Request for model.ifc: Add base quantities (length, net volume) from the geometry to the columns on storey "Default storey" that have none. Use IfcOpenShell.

First a look at what the model holds.

```python
import ifcopenshell
import ifcopenshell.util.element
import ifcopenshell.util.unit

model = ifcopenshell.open("model.ifc")
print(model.schema)
for unit_type in ("LENGTHUNIT", "AREAUNIT", "VOLUMEUNIT"):
    print(unit_type, ifcopenshell.util.unit.calculate_unit_scale(model, unit_type))
storey = next(s for s in model.by_type("IfcBuildingStorey") if s.Name == "Default storey")
columns = [e for e in ifcopenshell.util.element.get_decomposition(storey) if e.is_a("IfcColumn")]
for e in sorted(columns, key=lambda e: e.id()):
    print(e.id(), e.is_a(), e.Name, list(ifcopenshell.util.element.get_psets(e, qtos_only=True)), sep=" | ")
```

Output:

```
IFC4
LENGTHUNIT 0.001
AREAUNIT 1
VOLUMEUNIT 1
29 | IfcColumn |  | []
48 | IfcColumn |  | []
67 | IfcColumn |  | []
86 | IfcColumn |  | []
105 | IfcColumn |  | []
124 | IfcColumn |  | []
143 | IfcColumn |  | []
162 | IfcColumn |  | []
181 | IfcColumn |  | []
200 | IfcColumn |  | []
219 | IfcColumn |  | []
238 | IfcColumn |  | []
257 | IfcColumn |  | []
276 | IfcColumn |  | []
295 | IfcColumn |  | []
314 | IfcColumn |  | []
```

```python
import ifcopenshell
import ifcopenshell.api.pset
import ifcopenshell.geom
import ifcopenshell.util.element
import ifcopenshell.util.shape
import ifcopenshell.util.unit

model = ifcopenshell.open("model.ifc")
unit_scale = ifcopenshell.util.unit.calculate_unit_scale(model)
volume_scale = ifcopenshell.util.unit.calculate_unit_scale(model, "VOLUMEUNIT")
settings = ifcopenshell.geom.settings()

storey = next(s for s in model.by_type("IfcBuildingStorey") if s.Name == "Default storey")
columns = [e for e in ifcopenshell.util.element.get_decomposition(storey) if e.is_a("IfcColumn")]

for e in sorted(columns, key=lambda e: e.id()):
    if ifcopenshell.util.element.get_psets(e, qtos_only=True, should_inherit=False):
        continue
    # Geometry comes back in metres, in the element's own axes.
    shape = ifcopenshell.geom.create_shape(settings, e)
    values = {
        "Length": ifcopenshell.util.shape.get_z(shape.geometry) / unit_scale,
        "NetVolume": ifcopenshell.util.shape.get_volume(shape.geometry) / volume_scale,
    }
    qto = ifcopenshell.api.pset.add_qto(model, product=e, name="Qto_ColumnBaseQuantities")
    ifcopenshell.api.pset.edit_qto(model, qto=qto, properties=values)
    print(e.id(), {k: round(v, 3) for k, v in values.items()})

model.write("model-out.ifc")
```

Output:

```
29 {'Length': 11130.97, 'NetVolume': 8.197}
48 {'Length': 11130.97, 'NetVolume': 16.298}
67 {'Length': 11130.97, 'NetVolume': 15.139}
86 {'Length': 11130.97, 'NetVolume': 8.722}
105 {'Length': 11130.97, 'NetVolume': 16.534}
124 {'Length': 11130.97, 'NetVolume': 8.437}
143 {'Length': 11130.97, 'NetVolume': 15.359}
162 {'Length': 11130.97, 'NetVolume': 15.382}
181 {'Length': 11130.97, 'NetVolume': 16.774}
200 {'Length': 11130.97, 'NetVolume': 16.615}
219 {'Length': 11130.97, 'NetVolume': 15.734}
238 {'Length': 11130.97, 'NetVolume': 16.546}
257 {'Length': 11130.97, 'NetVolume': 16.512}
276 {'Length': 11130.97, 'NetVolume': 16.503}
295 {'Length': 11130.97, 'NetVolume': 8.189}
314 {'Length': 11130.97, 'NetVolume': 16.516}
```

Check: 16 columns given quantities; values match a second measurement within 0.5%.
